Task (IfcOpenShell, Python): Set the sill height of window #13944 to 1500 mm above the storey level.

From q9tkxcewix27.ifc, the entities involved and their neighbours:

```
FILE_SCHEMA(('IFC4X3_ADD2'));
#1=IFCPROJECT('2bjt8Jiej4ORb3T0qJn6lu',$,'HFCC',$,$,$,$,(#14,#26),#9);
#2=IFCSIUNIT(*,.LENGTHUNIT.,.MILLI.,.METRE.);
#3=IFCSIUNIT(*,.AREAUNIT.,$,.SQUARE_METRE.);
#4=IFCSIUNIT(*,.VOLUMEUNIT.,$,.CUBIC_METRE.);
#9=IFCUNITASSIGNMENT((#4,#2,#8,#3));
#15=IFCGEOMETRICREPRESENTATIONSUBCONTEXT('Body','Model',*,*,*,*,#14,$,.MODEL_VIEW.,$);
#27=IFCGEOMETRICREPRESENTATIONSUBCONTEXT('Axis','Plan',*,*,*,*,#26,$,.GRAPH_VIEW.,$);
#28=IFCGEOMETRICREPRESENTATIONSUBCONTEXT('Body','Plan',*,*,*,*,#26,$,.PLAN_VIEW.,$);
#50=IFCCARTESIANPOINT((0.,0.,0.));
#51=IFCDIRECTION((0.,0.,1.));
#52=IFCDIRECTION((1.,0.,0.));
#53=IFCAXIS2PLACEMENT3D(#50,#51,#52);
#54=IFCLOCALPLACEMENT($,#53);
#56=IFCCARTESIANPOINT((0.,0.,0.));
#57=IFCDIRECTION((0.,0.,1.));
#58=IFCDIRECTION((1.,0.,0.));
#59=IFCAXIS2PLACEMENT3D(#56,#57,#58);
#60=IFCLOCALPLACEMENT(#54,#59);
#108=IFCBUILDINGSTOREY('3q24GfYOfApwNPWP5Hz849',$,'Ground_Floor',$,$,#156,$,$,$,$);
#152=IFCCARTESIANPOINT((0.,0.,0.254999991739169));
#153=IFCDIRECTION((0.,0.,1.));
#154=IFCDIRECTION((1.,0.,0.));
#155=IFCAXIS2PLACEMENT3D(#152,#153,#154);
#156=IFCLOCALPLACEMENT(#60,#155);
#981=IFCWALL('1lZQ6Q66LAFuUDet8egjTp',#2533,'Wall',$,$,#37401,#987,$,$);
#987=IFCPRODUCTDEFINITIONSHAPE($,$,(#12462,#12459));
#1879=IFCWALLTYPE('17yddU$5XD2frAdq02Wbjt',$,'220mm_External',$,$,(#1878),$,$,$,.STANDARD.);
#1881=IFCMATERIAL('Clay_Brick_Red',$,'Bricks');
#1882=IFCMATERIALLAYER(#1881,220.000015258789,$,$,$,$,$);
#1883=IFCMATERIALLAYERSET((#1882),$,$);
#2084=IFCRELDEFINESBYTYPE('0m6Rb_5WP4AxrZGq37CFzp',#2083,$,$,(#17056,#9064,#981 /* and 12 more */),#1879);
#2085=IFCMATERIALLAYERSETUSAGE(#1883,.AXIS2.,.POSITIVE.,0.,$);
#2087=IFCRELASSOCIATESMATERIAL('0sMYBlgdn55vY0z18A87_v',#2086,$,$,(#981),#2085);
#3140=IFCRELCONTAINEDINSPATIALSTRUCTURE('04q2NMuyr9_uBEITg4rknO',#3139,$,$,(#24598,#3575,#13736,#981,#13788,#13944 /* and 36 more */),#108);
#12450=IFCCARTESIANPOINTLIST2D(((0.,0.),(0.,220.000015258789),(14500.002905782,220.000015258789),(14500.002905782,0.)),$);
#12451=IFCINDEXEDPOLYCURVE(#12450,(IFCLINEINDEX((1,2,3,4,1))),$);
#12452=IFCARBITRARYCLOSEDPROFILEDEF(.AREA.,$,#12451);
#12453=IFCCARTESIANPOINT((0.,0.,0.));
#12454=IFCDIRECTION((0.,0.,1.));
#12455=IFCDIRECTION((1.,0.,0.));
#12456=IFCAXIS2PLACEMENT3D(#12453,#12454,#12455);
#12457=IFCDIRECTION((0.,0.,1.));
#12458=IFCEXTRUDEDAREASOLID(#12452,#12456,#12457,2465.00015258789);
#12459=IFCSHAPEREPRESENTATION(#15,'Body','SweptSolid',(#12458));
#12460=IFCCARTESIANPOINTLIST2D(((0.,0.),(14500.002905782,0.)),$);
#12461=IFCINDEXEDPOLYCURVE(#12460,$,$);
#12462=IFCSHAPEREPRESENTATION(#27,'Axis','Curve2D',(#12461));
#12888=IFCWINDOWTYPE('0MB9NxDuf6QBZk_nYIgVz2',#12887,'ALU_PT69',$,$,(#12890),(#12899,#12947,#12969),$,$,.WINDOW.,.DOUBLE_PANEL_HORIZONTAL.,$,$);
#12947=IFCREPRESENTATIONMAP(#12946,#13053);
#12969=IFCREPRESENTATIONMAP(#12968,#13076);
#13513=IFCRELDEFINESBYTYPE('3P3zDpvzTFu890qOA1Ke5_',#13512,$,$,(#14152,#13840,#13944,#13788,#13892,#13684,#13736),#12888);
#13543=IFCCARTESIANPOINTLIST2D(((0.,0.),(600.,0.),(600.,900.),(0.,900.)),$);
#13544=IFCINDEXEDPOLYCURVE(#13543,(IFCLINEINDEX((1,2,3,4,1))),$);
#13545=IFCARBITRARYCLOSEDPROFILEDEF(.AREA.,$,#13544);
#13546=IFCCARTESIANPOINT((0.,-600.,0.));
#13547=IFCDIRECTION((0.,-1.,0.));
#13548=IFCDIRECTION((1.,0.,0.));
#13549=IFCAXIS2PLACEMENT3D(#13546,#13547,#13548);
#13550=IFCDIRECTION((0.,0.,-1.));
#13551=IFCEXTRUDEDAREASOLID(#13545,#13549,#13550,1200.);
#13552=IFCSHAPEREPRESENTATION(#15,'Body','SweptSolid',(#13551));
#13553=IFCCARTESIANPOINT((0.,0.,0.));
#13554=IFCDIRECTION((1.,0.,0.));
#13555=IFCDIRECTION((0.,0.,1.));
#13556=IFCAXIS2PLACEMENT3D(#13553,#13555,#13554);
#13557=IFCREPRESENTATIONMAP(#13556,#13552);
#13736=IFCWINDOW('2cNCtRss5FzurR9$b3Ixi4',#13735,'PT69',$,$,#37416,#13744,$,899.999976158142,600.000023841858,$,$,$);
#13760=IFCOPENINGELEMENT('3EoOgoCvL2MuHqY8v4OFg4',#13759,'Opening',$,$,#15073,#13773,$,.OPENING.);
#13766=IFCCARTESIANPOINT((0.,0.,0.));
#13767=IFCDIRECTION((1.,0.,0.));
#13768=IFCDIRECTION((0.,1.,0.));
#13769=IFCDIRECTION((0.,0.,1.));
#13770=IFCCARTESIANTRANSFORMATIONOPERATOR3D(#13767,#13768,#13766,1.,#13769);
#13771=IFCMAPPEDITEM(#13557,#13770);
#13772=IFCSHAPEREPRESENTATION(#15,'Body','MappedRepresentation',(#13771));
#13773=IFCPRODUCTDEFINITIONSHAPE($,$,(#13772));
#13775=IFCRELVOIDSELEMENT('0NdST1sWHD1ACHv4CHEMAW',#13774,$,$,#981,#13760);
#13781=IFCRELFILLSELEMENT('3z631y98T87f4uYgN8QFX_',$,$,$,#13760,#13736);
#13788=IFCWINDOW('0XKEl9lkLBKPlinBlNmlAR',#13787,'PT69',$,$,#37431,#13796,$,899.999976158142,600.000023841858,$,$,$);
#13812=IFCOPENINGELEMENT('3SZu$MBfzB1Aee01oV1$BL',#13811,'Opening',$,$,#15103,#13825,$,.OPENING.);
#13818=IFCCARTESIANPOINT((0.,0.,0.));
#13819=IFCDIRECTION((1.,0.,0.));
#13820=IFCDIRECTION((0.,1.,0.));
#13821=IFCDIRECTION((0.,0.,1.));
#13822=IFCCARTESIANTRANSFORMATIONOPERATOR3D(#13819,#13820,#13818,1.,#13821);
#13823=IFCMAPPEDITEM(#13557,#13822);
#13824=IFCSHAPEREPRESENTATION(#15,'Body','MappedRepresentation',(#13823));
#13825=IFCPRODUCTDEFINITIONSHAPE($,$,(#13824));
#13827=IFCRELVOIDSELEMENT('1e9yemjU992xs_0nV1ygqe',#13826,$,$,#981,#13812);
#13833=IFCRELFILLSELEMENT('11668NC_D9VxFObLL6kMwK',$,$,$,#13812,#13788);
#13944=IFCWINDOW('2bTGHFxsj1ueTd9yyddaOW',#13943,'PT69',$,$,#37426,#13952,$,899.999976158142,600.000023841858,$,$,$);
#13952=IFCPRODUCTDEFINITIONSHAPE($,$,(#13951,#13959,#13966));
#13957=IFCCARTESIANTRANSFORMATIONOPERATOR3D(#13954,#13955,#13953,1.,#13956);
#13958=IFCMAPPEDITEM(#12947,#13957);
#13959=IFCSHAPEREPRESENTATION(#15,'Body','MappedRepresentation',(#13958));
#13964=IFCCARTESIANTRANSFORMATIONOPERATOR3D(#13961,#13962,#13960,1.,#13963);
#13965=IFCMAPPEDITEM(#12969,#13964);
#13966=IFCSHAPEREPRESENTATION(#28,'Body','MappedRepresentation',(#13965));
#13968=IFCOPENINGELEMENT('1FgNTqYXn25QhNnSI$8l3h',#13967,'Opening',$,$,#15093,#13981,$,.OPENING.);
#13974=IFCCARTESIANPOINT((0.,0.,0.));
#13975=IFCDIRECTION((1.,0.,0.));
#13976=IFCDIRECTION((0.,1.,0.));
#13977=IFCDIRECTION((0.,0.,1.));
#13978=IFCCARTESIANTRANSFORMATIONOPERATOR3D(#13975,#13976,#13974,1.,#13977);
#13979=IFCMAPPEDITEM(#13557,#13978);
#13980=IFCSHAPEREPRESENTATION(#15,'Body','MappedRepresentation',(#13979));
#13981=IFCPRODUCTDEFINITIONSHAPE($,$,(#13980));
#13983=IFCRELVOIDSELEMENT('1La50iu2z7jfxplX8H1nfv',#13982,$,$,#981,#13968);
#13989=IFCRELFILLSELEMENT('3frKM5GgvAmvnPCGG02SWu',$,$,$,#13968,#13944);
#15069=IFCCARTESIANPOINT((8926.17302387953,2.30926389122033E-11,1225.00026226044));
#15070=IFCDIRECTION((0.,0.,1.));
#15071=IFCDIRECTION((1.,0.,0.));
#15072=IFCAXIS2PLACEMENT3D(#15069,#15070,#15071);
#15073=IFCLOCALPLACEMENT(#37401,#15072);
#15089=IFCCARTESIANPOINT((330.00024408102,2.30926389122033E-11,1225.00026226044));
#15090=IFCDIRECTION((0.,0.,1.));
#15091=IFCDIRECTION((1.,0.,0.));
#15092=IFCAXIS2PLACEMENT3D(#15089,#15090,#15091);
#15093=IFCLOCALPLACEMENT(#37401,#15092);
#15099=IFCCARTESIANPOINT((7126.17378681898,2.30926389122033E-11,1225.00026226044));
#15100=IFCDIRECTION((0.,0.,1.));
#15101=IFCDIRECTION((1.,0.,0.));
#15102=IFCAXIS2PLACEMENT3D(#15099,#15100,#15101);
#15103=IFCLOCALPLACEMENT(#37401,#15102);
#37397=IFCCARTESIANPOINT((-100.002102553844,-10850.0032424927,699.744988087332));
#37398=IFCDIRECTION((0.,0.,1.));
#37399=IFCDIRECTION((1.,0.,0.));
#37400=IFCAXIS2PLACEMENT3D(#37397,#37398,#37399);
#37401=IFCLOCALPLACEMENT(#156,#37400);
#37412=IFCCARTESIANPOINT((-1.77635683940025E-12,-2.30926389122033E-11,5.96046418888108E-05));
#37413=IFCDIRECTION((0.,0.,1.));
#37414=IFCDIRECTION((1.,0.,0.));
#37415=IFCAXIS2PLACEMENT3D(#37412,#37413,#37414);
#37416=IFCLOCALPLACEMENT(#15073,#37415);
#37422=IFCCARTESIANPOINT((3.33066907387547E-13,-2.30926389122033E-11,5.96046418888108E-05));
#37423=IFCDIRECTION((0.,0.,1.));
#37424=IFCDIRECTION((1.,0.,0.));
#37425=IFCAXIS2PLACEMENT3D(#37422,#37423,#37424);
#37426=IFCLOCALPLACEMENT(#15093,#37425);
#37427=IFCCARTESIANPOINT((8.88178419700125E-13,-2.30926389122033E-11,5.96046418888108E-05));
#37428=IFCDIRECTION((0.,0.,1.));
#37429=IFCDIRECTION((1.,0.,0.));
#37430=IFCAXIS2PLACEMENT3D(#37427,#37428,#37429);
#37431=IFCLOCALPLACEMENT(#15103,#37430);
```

```python
import numpy as np
import ifcopenshell
import ifcopenshell.api.geometry
import ifcopenshell.geom
import ifcopenshell.util.element
import ifcopenshell.util.placement
import ifcopenshell.util.shape
import ifcopenshell.util.unit

model = ifcopenshell.open("q9tkxcewix27.ifc")
unit_scale = ifcopenshell.util.unit.calculate_unit_scale(model)

window = model.by_id(13944)
opening = window.FillsVoids[0].RelatingOpeningElement
storey = ifcopenshell.util.element.get_container(window, ifc_class="IfcBuildingStorey")
level = ifcopenshell.util.placement.get_local_placement(storey.ObjectPlacement)[2, 3]

# The opening's origin need not be at the sill, so measure its lowest point.
shape = ifcopenshell.geom.create_shape(ifcopenshell.geom.settings(), opening)
bottom = ifcopenshell.util.shape.get_shape_bottom_elevation(shape, shape.geometry) / unit_scale
dz = level + 1.5 / unit_scale - bottom

shift = np.array([0.0, 0.0, dz])
# The window is placed relative to its opening, so it follows when the opening moves.
matrix = ifcopenshell.util.placement.get_local_placement(opening.ObjectPlacement)
matrix[:3, 3] += shift
ifcopenshell.api.geometry.edit_object_placement(
    model, product=opening, matrix=matrix, is_si=False, should_transform_children=True
)

print(f"moved by {dz * unit_scale:+.3f} m")

model.write("q9tkxcewix27_v2.ifc")
```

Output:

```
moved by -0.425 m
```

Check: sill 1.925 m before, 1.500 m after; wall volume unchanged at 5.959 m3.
